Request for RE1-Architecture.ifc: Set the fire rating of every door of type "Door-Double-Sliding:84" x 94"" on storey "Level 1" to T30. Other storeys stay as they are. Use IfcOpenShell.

First a look at what the model holds.

```python
import ifcopenshell
import ifcopenshell.util.element

model = ifcopenshell.open("RE1-Architecture.ifc")
print(model.schema)
storey = next(s for s in model.by_type("IfcBuildingStorey") if s.Name == "Level 1")
doors = [e for e in ifcopenshell.util.element.get_decomposition(storey) if e.is_a("IfcDoor")]
seen = {}
for e in doors:
    element_type = ifcopenshell.util.element.get_type(e)
    key = (element_type.Name if element_type != e and element_type else None, ifcopenshell.util.element.get_pset(e, "Pset_DoorCommon", "FireRating"))
    seen[key] = seen.get(key, 0) + 1
for (name, value), count in sorted(seen.items(), key=str):
    print(count, "x", name, "|", value)
```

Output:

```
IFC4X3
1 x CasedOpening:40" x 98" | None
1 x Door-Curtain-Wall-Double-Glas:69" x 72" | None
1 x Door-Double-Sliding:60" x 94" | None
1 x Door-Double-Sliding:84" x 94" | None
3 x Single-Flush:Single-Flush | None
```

```python
import ifcopenshell
import ifcopenshell.api.pset
import ifcopenshell.util.element

model = ifcopenshell.open("RE1-Architecture.ifc")

storey = next(s for s in model.by_type("IfcBuildingStorey") if s.Name == "Level 1")
doors = [e for e in ifcopenshell.util.element.get_decomposition(storey) if e.is_a("IfcDoor")]

count = 0
for e in doors:
    element_type = ifcopenshell.util.element.get_type(e)
    if element_type in (None, e) or element_type.Name != 'Door-Double-Sliding:84" x 94"':
        continue
    # add_pset returns the element's existing set when there is one.
    pset = ifcopenshell.api.pset.add_pset(model, product=e, name="Pset_DoorCommon")
    ifcopenshell.api.pset.edit_pset(model, pset=pset, properties={"FireRating": "T30"})
    count += 1

print(count, "doors updated")

model.write("RE1-Architecture-out.ifc")
```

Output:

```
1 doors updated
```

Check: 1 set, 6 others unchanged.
